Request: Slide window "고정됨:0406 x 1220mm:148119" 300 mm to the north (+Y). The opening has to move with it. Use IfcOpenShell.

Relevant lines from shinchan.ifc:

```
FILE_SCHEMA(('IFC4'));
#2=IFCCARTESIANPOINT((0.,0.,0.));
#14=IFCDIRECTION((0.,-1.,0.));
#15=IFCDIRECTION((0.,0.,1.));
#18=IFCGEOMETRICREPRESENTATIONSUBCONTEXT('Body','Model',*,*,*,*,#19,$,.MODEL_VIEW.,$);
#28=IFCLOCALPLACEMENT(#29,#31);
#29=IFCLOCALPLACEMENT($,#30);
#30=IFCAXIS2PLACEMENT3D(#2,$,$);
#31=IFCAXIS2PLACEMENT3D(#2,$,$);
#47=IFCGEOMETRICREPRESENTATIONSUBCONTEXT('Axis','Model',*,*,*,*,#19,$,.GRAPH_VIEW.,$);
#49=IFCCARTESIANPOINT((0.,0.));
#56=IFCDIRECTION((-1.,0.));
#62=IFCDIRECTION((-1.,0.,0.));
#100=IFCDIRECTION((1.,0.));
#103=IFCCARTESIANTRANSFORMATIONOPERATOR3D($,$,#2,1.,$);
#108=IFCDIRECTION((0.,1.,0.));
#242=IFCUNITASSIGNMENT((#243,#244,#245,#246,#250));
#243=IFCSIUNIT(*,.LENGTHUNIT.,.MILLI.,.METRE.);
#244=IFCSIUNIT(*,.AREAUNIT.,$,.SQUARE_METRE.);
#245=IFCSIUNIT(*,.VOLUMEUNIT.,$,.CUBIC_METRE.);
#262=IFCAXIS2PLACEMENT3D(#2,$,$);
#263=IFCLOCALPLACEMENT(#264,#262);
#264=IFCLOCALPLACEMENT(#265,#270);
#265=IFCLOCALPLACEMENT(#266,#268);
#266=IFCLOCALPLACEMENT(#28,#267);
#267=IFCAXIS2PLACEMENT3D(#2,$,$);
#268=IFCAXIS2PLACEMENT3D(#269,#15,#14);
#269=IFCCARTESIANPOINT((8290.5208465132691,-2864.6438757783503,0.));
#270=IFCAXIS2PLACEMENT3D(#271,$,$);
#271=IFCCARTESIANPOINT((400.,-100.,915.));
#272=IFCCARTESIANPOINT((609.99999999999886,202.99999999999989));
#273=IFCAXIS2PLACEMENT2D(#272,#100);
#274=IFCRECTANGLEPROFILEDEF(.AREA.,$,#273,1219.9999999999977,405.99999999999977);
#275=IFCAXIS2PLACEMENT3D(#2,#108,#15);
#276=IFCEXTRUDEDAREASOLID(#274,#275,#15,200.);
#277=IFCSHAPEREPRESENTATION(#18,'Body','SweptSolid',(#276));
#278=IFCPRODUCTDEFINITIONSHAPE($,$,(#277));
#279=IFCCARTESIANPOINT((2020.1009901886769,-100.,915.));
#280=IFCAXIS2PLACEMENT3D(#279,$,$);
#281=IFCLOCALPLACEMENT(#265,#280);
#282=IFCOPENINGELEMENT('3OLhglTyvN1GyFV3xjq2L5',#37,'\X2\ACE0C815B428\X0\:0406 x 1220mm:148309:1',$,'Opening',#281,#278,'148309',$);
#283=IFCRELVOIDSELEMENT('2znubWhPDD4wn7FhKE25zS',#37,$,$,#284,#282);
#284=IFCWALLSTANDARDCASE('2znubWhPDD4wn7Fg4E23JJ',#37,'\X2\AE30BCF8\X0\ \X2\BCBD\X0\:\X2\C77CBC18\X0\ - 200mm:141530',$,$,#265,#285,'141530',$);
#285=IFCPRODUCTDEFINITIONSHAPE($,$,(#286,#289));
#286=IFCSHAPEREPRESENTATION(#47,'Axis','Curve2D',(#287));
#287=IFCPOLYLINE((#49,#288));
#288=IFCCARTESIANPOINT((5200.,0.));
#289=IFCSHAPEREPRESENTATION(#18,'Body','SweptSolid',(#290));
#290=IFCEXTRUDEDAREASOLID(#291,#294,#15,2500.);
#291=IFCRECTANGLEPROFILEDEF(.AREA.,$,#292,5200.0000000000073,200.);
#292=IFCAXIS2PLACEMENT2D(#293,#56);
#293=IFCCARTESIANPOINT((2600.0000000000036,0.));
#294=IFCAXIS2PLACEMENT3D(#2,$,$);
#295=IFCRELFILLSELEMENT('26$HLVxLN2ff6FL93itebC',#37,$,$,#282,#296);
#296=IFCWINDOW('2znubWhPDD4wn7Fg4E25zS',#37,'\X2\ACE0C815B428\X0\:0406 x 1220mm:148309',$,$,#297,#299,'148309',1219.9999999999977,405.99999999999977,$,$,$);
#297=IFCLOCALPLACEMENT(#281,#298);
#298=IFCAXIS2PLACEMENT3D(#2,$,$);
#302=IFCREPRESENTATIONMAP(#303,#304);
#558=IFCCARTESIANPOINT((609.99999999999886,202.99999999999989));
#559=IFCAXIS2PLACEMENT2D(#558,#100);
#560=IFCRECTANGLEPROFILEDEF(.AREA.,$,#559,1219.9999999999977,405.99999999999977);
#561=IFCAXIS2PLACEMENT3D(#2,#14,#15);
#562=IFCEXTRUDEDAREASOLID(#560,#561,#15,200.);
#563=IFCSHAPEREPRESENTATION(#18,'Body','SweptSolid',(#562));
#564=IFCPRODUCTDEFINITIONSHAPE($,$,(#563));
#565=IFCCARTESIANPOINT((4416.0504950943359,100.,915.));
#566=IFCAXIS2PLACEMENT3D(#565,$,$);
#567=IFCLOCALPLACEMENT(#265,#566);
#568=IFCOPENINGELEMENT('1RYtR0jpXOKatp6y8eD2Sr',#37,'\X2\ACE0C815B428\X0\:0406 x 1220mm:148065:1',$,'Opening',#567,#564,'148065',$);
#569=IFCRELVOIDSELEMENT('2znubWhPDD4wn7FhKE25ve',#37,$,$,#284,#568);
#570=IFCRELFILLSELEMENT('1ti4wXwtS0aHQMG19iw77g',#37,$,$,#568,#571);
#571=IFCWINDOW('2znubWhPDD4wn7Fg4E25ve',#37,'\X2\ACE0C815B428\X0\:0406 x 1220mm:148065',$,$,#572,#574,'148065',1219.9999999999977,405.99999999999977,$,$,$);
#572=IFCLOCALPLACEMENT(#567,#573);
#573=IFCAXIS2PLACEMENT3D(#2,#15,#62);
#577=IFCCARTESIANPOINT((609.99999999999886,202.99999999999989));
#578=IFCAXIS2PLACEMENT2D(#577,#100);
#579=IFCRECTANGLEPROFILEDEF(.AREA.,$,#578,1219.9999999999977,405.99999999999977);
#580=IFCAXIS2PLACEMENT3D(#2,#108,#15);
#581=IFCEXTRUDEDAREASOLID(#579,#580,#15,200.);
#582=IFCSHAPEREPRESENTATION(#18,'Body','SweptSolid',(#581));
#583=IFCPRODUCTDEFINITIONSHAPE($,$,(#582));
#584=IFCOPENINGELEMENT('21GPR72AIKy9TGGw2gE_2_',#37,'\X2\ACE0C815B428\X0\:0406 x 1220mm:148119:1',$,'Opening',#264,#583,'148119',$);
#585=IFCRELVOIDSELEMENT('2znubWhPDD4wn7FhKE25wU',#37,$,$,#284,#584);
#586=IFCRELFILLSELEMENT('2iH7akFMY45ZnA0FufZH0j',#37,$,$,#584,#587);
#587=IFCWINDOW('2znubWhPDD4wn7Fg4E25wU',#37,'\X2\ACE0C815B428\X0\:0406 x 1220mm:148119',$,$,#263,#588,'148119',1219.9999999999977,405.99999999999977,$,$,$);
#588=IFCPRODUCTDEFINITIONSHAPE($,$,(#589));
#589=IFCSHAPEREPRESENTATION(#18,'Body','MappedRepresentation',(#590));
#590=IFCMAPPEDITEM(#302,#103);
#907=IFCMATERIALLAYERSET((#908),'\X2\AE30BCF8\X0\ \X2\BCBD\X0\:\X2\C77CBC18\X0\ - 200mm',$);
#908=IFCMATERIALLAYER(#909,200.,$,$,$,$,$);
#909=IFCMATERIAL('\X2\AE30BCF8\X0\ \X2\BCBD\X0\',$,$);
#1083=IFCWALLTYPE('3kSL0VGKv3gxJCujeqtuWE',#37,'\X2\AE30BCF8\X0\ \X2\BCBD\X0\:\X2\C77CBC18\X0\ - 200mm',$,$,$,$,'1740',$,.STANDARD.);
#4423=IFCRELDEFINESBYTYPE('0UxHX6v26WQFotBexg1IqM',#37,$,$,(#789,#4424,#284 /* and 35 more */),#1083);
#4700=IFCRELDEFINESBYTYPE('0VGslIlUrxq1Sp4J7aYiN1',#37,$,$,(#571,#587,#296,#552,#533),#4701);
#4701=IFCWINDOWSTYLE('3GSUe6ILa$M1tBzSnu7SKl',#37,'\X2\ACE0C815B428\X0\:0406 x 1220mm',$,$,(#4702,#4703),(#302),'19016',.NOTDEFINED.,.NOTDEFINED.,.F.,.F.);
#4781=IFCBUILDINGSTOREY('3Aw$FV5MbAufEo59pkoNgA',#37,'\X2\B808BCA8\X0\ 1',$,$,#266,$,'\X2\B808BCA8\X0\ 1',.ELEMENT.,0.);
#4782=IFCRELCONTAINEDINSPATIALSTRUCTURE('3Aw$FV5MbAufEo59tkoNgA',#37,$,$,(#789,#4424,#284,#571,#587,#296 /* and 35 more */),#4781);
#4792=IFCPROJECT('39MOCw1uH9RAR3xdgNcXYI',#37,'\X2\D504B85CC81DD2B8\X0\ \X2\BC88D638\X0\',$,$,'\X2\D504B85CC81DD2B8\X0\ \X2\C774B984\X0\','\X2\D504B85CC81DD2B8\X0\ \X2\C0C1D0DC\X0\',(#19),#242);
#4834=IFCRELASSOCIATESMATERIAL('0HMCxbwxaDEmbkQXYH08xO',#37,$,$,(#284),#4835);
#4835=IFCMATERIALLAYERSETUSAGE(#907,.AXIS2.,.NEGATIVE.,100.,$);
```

```python
import ifcopenshell
import ifcopenshell.api.geometry
import ifcopenshell.util.placement
import ifcopenshell.util.unit

model = ifcopenshell.open("shinchan.ifc")
unit_scale = ifcopenshell.util.unit.calculate_unit_scale(model)

window = model.by_guid("2znubWhPDD4wn7Fg4E25wU")
opening = window.FillsVoids[0].RelatingOpeningElement
wall = opening.VoidsElements[0].RelatingBuildingElement

wall_matrix = ifcopenshell.util.placement.get_local_placement(wall.ObjectPlacement)
shift = wall_matrix[:3, 0] * -0.3 / unit_scale
before = ifcopenshell.util.placement.get_local_placement(window.ObjectPlacement)[:3, 3].copy()

# The window is placed relative to its opening, so it follows when the opening moves.
matrix = ifcopenshell.util.placement.get_local_placement(opening.ObjectPlacement)
matrix[:3, 3] += shift
ifcopenshell.api.geometry.edit_object_placement(
    model, product=opening, matrix=matrix, is_si=False, should_transform_children=True
)

after = ifcopenshell.util.placement.get_local_placement(window.ObjectPlacement)[:3, 3]
print("window moved by", (after - before).round(3) + 0.0)

model.write("shinchan_edited.ifc")
```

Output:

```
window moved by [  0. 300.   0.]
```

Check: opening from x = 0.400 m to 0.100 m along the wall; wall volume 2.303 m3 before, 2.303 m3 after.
